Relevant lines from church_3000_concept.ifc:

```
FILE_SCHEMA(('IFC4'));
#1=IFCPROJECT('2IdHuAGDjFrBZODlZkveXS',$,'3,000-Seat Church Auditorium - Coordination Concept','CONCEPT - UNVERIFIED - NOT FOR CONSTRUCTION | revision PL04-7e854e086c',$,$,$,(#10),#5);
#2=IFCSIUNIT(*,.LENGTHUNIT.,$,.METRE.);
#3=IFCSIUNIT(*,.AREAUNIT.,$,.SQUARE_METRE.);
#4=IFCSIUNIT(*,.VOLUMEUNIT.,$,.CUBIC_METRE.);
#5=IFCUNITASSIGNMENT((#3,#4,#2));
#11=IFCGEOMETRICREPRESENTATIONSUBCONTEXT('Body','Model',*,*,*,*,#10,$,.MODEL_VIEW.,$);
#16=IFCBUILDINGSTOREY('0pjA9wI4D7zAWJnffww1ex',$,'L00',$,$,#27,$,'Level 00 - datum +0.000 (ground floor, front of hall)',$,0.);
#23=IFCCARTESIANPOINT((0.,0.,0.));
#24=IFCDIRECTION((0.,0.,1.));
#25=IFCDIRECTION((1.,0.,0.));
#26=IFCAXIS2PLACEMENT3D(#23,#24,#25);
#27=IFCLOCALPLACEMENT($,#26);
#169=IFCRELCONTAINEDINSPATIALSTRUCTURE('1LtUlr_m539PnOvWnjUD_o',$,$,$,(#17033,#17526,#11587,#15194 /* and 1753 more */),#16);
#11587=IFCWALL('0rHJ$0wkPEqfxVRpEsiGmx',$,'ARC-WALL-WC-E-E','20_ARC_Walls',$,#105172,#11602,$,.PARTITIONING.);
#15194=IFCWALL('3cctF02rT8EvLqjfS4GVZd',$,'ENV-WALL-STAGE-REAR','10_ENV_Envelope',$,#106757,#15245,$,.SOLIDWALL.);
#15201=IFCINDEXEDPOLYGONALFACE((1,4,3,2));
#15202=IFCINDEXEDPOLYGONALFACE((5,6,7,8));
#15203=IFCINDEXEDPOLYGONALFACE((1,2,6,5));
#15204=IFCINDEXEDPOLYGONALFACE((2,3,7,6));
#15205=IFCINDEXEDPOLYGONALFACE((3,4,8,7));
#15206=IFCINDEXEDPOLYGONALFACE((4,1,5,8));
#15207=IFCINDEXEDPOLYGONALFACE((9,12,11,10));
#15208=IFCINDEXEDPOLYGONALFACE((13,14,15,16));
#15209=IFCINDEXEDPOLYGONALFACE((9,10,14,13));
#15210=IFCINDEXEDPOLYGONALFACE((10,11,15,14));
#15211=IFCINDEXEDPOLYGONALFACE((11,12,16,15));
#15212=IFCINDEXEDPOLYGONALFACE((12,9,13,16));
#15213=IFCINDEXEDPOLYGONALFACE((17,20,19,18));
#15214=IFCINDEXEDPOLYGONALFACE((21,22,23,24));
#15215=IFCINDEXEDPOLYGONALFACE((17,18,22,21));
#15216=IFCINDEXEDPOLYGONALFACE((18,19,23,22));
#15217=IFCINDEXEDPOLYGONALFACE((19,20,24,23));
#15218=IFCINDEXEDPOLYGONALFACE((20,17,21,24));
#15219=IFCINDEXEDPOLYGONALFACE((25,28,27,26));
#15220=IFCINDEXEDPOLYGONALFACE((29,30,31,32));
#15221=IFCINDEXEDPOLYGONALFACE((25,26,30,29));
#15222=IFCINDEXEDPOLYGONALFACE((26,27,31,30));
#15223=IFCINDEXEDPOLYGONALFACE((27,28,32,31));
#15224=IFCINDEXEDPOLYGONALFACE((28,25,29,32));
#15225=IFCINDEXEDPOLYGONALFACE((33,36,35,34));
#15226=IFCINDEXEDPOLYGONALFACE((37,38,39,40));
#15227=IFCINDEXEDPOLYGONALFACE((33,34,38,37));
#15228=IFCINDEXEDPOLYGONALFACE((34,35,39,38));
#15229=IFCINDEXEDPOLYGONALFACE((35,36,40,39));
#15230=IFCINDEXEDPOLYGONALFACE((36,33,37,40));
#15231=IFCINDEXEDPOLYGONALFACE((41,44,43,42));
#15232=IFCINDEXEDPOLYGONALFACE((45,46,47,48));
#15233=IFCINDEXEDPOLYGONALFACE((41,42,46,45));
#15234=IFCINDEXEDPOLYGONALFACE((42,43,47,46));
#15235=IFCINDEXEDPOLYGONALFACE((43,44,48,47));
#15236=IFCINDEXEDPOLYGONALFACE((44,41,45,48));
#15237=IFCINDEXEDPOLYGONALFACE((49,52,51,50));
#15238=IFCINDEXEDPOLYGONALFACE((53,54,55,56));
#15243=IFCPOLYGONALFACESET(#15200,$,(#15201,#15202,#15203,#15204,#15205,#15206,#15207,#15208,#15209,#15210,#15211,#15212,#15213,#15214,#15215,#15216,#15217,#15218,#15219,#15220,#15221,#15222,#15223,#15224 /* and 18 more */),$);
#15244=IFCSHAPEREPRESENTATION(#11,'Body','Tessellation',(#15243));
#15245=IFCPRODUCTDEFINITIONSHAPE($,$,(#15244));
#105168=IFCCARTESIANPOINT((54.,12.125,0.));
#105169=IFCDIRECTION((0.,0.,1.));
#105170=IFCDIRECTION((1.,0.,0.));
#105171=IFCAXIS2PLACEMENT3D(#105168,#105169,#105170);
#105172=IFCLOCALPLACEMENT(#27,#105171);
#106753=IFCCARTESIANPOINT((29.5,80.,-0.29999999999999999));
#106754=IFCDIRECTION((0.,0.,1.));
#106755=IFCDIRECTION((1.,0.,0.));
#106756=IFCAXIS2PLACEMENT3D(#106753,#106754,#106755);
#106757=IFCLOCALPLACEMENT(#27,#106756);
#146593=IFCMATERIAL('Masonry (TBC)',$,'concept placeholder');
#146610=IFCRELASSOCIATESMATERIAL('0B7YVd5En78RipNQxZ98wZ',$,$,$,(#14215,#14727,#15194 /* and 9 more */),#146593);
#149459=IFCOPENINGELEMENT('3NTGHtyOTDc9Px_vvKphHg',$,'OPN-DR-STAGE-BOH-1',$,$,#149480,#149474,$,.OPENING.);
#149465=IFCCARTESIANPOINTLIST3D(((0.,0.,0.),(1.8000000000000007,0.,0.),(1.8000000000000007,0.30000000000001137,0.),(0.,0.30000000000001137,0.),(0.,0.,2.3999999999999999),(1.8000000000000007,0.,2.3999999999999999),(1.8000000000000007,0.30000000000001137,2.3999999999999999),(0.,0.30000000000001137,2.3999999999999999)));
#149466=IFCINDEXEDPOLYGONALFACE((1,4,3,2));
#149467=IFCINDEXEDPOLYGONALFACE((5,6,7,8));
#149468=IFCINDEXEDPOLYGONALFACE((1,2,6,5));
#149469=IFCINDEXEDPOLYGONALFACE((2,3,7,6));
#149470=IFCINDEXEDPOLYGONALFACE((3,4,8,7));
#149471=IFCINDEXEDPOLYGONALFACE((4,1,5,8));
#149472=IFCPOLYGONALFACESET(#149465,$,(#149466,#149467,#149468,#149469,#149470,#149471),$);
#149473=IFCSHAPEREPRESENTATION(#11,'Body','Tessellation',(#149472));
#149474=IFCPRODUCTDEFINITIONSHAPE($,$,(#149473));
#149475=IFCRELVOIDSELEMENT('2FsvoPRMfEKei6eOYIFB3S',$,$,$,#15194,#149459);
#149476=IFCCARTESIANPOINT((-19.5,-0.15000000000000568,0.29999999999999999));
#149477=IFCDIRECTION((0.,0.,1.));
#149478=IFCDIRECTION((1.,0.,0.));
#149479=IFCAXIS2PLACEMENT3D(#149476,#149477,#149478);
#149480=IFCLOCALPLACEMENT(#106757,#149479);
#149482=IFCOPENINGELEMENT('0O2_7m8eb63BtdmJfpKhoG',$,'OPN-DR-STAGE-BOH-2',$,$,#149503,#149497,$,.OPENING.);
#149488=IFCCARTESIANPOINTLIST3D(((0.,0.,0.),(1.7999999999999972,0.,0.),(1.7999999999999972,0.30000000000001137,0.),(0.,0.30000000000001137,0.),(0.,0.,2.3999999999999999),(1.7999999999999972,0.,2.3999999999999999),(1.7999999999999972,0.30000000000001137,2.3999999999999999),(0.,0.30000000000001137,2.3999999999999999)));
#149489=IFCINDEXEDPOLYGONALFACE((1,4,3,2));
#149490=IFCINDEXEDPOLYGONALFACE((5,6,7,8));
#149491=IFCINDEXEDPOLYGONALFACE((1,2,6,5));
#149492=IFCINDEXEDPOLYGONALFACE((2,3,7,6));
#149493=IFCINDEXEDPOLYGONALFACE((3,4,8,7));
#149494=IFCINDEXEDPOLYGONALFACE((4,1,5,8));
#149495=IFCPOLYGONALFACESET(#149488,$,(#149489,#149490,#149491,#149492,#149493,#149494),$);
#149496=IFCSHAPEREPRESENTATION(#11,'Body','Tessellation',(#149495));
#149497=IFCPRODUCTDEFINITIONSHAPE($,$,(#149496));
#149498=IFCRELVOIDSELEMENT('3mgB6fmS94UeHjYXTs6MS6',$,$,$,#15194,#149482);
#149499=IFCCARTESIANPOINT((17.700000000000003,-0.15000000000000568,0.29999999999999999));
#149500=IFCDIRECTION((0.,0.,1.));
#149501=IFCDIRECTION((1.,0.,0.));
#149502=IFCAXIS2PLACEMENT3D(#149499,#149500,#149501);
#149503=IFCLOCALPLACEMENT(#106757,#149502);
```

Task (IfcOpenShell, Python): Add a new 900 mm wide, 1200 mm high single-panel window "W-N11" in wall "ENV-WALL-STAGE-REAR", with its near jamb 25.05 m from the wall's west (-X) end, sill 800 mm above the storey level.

```python
import numpy as np
import ifcopenshell
import ifcopenshell.api.feature
import ifcopenshell.api.geometry
import ifcopenshell.api.root
import ifcopenshell.api.spatial
import ifcopenshell.geom
import ifcopenshell.util.element
import ifcopenshell.util.placement
import ifcopenshell.util.representation
import ifcopenshell.util.shape
import ifcopenshell.util.unit

model = ifcopenshell.open("church_3000_concept.ifc")
unit_scale = ifcopenshell.util.unit.calculate_unit_scale(model)
settings = ifcopenshell.geom.settings()


def volume(element):
    """Net volume in cubic metres, openings subtracted."""
    shape = ifcopenshell.geom.create_shape(settings, element)
    return ifcopenshell.util.shape.get_volume(shape.geometry)


wall = model.by_guid("3cctF02rT8EvLqjfS4GVZd")
storey = ifcopenshell.util.element.get_container(wall, ifc_class="IfcBuildingStorey")
context = ifcopenshell.util.representation.get_context(model, "Model", "Body", "MODEL_VIEW")
before = volume(wall)

width, height, from_end, sill = 0.9, 1.2, 25.05, 0.8  # metres

# The wall runs along its own X axis, and the end named is its -X end.
wall_shape = ifcopenshell.geom.create_shape(settings, wall)
x, y, z = ifcopenshell.util.shape.get_vertices(wall_shape.geometry).T
start = x.min() + from_end
face, thickness = float(y.min()), float(y.max() - y.min())
wall_matrix = ifcopenshell.util.placement.get_local_placement(wall.ObjectPlacement)
level = ifcopenshell.util.placement.get_local_placement(storey.ObjectPlacement)[2, 3]


def in_wall(x, y):
    """Placement at x, y metres in the wall's axes, at sill height."""
    matrix = wall_matrix.copy()
    matrix[:, 3] = wall_matrix @ np.array([x / unit_scale, y / unit_scale, 0.0, 1.0])
    matrix[2, 3] = level + sill / unit_scale
    return matrix


# Opening: a box that overshoots both wall faces by 50 mm.
opening = ifcopenshell.api.root.create_entity(model, ifc_class="IfcOpeningElement", predefined_type="OPENING")
box = ifcopenshell.api.geometry.add_wall_representation(
    model, context=context, length=width, height=height, thickness=thickness + 0.1
)
ifcopenshell.api.geometry.assign_representation(model, product=opening, representation=box)
ifcopenshell.api.geometry.edit_object_placement(model, product=opening, matrix=in_wall(start, face - 0.05), is_si=False)
ifcopenshell.api.feature.add_feature(model, feature=opening, element=wall)

window = ifcopenshell.api.root.create_entity(model, ifc_class="IfcWindow", name="W-N11", predefined_type="WINDOW")
window.OverallWidth, window.OverallHeight = width / unit_scale, height / unit_scale
window.PartitioningType = "SINGLE_PANEL"
body = ifcopenshell.api.geometry.add_window_representation(
    model,
    context=context,
    overall_width=window.OverallWidth,
    overall_height=window.OverallHeight,
    partition_type="SINGLE_PANEL",
)
ifcopenshell.api.geometry.assign_representation(model, product=window, representation=body)
ifcopenshell.api.spatial.assign_container(model, products=[window], relating_structure=storey)
ifcopenshell.api.feature.add_filling(model, opening=opening, element=window)

# Centre the window in the wall's thickness.
ifcopenshell.api.geometry.edit_object_placement(model, product=window, matrix=in_wall(start, face), is_si=False)
window_shape = ifcopenshell.geom.create_shape(settings, window)
depth = ifcopenshell.util.shape.get_vertices(window_shape.geometry)[:, 1]
offset = face + thickness / 2 - (depth.min() + depth.max()) / 2
ifcopenshell.api.geometry.edit_object_placement(model, product=window, matrix=in_wall(start, offset), is_si=False)

after = volume(wall)

print(f"wall volume {before:.3f} -> {after:.3f} m3")

model.write("church_3000_concept_updated.ifc")
```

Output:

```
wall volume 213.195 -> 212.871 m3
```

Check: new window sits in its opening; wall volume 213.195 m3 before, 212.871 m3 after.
